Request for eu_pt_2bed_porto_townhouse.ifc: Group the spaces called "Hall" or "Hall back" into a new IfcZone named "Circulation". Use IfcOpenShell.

First a look at what the model holds.

```python
import ifcopenshell

model = ifcopenshell.open("eu_pt_2bed_porto_townhouse.ifc")
print(model.schema)
seen = {}
for space in model.by_type("IfcSpace"):
    seen[space.LongName] = seen.get(space.LongName, 0) + 1
for name, count in sorted(seen.items(), key=str):
    print(count, "x", name)
print("zones:", [z.Name for z in model.by_type("IfcZone")][:20])
```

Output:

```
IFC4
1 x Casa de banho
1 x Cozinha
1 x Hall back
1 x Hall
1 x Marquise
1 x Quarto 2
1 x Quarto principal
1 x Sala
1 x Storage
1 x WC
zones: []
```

```python
import ifcopenshell
import ifcopenshell.api.group
import ifcopenshell.api.root

model = ifcopenshell.open("eu_pt_2bed_porto_townhouse.ifc")

names = {"Hall", "Hall back"}
spaces = [s for s in model.by_type("IfcSpace") if s.LongName in names]

zone = ifcopenshell.api.root.create_entity(model, ifc_class="IfcZone", name="Circulation")
ifcopenshell.api.group.assign_group(model, products=spaces, group=zone)
print(len(spaces), "spaces in", zone.Name)

model.write("eu_pt_2bed_porto_townhouse-out.ifc")
```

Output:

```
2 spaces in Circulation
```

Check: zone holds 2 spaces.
